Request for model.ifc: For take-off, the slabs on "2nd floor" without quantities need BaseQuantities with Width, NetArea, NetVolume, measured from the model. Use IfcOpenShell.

First a look at what the model holds.

```python
import ifcopenshell
import ifcopenshell.util.element
import ifcopenshell.util.unit

model = ifcopenshell.open("model.ifc")
print(model.schema)
for unit_type in ("LENGTHUNIT", "AREAUNIT", "VOLUMEUNIT"):
    print(unit_type, ifcopenshell.util.unit.calculate_unit_scale(model, unit_type))
storey = next(s for s in model.by_type("IfcBuildingStorey") if s.Name == "2nd floor")
slabs = [e for e in ifcopenshell.util.element.get_decomposition(storey) if e.is_a("IfcSlab")]
for e in sorted(slabs, key=lambda e: e.id()):
    print(e.id(), e.is_a(), e.Name, list(ifcopenshell.util.element.get_psets(e, qtos_only=True)), sep=" | ")
```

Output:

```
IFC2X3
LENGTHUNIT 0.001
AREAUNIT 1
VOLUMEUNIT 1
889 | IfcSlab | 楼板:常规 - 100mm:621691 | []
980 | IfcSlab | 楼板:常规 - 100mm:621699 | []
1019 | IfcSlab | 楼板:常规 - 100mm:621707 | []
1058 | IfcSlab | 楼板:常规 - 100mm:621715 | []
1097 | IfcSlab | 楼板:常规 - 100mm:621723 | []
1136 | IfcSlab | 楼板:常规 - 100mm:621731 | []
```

```python
import ifcopenshell
import ifcopenshell.api.pset
import ifcopenshell.geom
import ifcopenshell.util.element
import ifcopenshell.util.shape
import ifcopenshell.util.unit

model = ifcopenshell.open("model.ifc")
unit_scale = ifcopenshell.util.unit.calculate_unit_scale(model)
area_scale = ifcopenshell.util.unit.calculate_unit_scale(model, "AREAUNIT")
volume_scale = ifcopenshell.util.unit.calculate_unit_scale(model, "VOLUMEUNIT")
settings = ifcopenshell.geom.settings()

storey = next(s for s in model.by_type("IfcBuildingStorey") if s.Name == "2nd floor")
slabs = [e for e in ifcopenshell.util.element.get_decomposition(storey) if e.is_a("IfcSlab")]

for e in sorted(slabs, key=lambda e: e.id()):
    if ifcopenshell.util.element.get_psets(e, qtos_only=True, should_inherit=False):
        continue
    # Geometry comes back in metres, in the element's own axes.
    shape = ifcopenshell.geom.create_shape(settings, e)
    values = {
        "Width": ifcopenshell.util.shape.get_z(shape.geometry) / unit_scale,
        "NetArea": ifcopenshell.util.shape.get_footprint_area(shape.geometry) / area_scale,
        "NetVolume": ifcopenshell.util.shape.get_volume(shape.geometry) / volume_scale,
    }
    qto = ifcopenshell.api.pset.add_qto(model, product=e, name="BaseQuantities")
    ifcopenshell.api.pset.edit_qto(model, qto=qto, properties=values)
    print(e.id(), {k: round(v, 3) for k, v in values.items()})

model.write("model_rev.ifc")
```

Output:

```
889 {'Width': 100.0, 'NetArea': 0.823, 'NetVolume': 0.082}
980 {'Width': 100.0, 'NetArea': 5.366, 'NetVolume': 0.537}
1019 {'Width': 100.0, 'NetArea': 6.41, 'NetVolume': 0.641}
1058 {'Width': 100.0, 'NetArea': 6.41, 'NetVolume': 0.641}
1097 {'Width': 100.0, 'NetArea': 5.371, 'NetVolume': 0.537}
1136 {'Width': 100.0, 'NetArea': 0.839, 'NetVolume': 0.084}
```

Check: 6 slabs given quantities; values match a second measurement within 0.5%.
